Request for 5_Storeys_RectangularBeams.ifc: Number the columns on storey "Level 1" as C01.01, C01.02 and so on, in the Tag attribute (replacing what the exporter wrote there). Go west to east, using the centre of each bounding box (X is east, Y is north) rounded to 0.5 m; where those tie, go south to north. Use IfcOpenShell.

First a look at what the model holds.

```python
import ifcopenshell
import ifcopenshell.util.element
import ifcopenshell.util.placement

model = ifcopenshell.open("5_Storeys_RectangularBeams.ifc")
print(model.schema)
storey = next(s for s in model.by_type("IfcBuildingStorey") if s.Name == "Level 1")
columns = [e for e in ifcopenshell.util.element.get_decomposition(storey) if e.is_a("IfcColumn")]
for e in sorted(columns, key=lambda e: e.id()):
    origin = ifcopenshell.util.placement.get_local_placement(e.ObjectPlacement)[:3, 3]
    print(e.id(), e.Tag, e.Name, origin.round(2) + 0.0, sep=" | ")
```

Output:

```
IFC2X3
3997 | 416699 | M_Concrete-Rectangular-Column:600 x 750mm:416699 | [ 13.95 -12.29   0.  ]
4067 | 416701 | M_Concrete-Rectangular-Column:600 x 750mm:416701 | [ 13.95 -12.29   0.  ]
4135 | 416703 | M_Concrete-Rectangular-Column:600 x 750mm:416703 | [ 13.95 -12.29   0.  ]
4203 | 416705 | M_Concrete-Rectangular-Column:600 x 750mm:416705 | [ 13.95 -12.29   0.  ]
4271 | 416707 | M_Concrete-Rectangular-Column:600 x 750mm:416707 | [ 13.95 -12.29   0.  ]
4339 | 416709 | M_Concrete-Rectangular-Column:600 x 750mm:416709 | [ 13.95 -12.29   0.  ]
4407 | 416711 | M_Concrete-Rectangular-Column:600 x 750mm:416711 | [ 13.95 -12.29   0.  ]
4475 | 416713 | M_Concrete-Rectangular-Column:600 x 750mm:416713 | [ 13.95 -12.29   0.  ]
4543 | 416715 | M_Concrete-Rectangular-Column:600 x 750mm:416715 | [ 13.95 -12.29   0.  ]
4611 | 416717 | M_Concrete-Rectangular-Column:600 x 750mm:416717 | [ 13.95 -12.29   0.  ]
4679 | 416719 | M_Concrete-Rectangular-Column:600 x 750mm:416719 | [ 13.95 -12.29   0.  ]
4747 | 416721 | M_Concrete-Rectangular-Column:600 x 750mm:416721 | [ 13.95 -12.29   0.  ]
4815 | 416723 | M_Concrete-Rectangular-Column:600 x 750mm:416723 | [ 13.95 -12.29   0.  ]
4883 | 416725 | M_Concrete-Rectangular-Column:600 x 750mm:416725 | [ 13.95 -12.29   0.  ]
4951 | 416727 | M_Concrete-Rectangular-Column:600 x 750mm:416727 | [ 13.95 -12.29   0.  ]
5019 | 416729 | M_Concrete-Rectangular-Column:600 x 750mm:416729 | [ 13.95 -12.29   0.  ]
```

```python
import ifcopenshell
import ifcopenshell.geom
import ifcopenshell.util.element
import ifcopenshell.util.shape

model = ifcopenshell.open("5_Storeys_RectangularBeams.ifc")
settings = ifcopenshell.geom.settings()
settings.set("use-world-coords", True)


def centre(element):
    shape = ifcopenshell.geom.create_shape(settings, element)
    return ifcopenshell.util.shape.get_bbox_centroid(shape.geometry)


storey = next(s for s in model.by_type("IfcBuildingStorey") if s.Name == "Level 1")
columns = [e for e in ifcopenshell.util.element.get_decomposition(storey) if e.is_a("IfcColumn")]

# Insertion points can sit at a corner or the storey origin, so sort by the geometry (in metres).
centres = {e: centre(e) for e in columns}
columns.sort(key=lambda e: (round(centres[e][0] / 0.5), centres[e][1]))

for i, e in enumerate(columns, start=1):
    number = f"C01.{i:02d}"
    e.Tag = number
    print(e.id(), number)

model.write("5_Storeys_RectangularBeams_v2.ifc")
```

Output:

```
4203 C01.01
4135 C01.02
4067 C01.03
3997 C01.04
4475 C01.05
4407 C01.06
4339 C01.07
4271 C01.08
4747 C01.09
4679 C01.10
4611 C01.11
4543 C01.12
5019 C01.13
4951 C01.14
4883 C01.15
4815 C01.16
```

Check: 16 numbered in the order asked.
